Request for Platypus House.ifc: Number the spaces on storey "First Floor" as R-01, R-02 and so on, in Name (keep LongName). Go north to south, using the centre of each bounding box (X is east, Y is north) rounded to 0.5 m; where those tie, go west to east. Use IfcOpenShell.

First a look at what the model holds.

```python
import ifcopenshell
import ifcopenshell.util.element
import ifcopenshell.util.placement

model = ifcopenshell.open("Platypus House.ifc")
print(model.schema)
storey = next(s for s in model.by_type("IfcBuildingStorey") if s.Name == "First Floor")
spaces = [e for e in ifcopenshell.util.element.get_decomposition(storey) if e.is_a("IfcSpace")]
for e in sorted(spaces, key=lambda e: e.id()):
    origin = ifcopenshell.util.placement.get_local_placement(e.ObjectPlacement)[:3, 3]
    print(e.id(), e.Name, e.LongName, origin.round(2) + 0.0, sep=" | ")
```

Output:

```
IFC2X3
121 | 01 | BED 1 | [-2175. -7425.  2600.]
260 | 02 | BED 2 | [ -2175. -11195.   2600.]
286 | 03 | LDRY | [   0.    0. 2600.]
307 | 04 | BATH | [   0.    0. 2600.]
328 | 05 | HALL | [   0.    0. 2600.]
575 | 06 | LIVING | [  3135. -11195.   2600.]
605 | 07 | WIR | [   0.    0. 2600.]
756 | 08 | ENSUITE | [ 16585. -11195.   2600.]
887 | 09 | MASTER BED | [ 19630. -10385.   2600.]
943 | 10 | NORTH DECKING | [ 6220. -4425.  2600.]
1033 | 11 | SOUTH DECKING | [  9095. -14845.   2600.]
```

```python
import ifcopenshell
import ifcopenshell.geom
import ifcopenshell.util.element
import ifcopenshell.util.shape

model = ifcopenshell.open("Platypus House.ifc")
settings = ifcopenshell.geom.settings()
settings.set("use-world-coords", True)


def centre(element):
    shape = ifcopenshell.geom.create_shape(settings, element)
    return ifcopenshell.util.shape.get_bbox_centroid(shape.geometry)


storey = next(s for s in model.by_type("IfcBuildingStorey") if s.Name == "First Floor")
spaces = [e for e in ifcopenshell.util.element.get_decomposition(storey) if e.is_a("IfcSpace")]

# Insertion points can sit at a corner or the storey origin, so sort by the geometry (in metres).
centres = {e: centre(e) for e in spaces}
spaces.sort(key=lambda e: (-round(centres[e][1] / 0.5), centres[e][0]))

for i, e in enumerate(spaces, start=1):
    number = f"R-{i:02d}"
    e.Name = number
    print(e.id(), number)

model.write("Platypus House_rev.ifc")
```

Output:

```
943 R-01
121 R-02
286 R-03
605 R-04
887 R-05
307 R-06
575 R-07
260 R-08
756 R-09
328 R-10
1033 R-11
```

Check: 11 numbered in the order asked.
